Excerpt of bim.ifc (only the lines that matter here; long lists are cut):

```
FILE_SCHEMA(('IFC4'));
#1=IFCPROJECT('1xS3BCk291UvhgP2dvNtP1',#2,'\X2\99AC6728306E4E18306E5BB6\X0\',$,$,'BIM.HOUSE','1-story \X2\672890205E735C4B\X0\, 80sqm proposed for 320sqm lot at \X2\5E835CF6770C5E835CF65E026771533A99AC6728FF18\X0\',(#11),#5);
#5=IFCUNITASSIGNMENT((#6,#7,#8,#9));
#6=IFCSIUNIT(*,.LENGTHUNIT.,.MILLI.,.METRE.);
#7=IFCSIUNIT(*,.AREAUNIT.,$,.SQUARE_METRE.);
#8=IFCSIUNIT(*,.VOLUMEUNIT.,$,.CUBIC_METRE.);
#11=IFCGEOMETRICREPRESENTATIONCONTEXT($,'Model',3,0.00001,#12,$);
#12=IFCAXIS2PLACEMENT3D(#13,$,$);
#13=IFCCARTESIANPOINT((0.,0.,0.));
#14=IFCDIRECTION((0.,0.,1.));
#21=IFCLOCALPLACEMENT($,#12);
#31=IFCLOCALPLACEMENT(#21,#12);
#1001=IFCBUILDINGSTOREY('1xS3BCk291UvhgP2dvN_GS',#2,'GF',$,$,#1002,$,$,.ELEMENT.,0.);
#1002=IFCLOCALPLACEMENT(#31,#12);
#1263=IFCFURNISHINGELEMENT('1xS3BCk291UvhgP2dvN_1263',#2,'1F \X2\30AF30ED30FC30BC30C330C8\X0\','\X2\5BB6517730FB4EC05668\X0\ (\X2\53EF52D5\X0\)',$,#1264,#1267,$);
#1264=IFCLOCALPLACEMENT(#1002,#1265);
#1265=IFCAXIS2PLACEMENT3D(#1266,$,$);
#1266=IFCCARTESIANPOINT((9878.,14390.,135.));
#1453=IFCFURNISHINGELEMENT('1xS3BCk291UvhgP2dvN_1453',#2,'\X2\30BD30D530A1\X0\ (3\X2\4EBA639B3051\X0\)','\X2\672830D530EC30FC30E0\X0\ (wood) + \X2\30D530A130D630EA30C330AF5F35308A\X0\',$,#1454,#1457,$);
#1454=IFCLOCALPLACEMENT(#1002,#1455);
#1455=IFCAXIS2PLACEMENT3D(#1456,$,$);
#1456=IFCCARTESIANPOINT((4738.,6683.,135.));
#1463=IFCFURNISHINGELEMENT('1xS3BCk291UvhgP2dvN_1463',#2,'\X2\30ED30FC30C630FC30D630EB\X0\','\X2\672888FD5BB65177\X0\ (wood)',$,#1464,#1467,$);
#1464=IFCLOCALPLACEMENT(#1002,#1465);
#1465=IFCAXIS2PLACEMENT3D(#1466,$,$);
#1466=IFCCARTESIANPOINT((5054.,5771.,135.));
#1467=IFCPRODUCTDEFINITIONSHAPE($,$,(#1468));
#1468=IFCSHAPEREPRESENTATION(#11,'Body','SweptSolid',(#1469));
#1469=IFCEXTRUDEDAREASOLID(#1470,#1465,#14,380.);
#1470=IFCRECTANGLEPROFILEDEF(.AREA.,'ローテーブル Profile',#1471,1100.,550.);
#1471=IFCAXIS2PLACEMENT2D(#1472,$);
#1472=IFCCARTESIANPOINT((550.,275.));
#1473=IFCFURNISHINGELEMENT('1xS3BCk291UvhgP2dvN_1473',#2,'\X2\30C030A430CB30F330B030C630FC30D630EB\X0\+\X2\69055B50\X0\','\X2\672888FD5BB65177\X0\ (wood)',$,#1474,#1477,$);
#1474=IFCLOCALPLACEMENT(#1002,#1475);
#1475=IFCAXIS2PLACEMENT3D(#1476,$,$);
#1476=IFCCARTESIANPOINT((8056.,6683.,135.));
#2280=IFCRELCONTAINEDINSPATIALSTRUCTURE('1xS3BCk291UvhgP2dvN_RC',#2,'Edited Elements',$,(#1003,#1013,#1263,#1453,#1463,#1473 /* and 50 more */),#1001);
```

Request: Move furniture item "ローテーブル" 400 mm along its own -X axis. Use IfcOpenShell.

```python
import ifcopenshell
import ifcopenshell.api.geometry
import ifcopenshell.util.placement
import ifcopenshell.util.unit

model = ifcopenshell.open("bim.ifc")
unit_scale = ifcopenshell.util.unit.calculate_unit_scale(model)

item = model.by_guid("1xS3BCk291UvhgP2dvN_1463")
matrix = ifcopenshell.util.placement.get_local_placement(item.ObjectPlacement)
matrix[:3, 3] -= matrix[:3, 0] * 0.4 / unit_scale
ifcopenshell.api.geometry.edit_object_placement(model, product=item, matrix=matrix, is_si=False)

print(ifcopenshell.util.placement.get_local_placement(item.ObjectPlacement).round(3) + 0.0)

model.write("bim_updated.ifc")
```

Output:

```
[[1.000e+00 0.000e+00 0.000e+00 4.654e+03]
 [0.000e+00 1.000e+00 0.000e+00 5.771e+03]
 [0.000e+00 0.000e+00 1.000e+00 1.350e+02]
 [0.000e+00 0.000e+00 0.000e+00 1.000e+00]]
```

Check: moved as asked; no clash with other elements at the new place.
